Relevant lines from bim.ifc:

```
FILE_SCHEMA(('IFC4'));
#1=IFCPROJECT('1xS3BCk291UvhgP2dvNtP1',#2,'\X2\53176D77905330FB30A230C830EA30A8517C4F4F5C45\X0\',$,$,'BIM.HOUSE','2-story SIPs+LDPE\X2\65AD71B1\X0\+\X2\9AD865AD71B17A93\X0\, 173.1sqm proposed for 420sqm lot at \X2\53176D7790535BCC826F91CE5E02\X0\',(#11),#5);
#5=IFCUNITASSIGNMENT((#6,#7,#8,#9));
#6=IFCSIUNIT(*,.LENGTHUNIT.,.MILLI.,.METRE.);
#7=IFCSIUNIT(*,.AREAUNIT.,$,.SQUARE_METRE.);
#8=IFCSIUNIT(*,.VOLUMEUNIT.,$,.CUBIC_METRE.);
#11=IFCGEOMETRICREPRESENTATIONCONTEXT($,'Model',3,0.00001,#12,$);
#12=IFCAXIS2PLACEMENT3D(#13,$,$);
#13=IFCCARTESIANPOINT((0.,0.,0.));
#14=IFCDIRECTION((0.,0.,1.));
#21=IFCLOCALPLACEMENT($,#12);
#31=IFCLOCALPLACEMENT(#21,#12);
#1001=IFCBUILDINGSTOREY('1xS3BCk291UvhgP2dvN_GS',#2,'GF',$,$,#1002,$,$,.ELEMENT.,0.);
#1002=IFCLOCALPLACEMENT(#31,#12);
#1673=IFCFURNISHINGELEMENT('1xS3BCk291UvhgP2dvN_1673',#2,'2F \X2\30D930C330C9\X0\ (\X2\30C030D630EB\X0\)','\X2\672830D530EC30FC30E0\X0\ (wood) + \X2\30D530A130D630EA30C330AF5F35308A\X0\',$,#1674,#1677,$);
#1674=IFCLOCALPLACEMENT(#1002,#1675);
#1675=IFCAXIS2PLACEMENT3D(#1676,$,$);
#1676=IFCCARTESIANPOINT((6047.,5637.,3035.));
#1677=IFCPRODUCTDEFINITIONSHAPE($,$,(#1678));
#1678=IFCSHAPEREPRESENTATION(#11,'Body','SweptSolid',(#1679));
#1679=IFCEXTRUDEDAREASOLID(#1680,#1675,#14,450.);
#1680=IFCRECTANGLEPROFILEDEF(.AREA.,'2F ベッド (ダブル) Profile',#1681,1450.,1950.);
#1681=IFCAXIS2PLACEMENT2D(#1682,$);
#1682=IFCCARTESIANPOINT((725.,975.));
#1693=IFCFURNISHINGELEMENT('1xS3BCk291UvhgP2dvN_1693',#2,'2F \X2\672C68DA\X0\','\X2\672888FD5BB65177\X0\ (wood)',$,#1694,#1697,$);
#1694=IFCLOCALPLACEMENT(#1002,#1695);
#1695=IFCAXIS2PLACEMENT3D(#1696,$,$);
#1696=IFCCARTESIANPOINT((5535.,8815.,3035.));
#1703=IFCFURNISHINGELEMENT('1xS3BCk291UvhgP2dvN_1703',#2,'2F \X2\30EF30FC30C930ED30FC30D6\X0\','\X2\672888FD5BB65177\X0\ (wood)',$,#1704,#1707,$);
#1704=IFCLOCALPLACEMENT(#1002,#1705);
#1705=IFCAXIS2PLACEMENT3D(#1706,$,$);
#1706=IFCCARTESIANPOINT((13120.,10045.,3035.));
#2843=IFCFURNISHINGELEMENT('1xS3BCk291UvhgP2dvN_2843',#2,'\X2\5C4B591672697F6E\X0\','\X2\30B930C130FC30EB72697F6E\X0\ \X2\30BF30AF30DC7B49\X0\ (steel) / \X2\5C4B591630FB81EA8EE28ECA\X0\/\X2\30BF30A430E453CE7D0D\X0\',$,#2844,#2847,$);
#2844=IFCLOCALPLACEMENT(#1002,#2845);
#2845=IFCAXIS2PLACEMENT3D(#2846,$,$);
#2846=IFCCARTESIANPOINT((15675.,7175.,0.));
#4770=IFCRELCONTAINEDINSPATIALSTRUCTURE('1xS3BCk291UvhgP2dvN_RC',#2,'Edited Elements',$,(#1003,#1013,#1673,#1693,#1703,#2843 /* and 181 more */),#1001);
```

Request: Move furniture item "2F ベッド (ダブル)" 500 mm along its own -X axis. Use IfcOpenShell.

```python
import ifcopenshell
import ifcopenshell.api.geometry
import ifcopenshell.util.placement

model = ifcopenshell.open("bim.ifc")

item = model.by_id(1673)
matrix = ifcopenshell.util.placement.get_local_placement(item.ObjectPlacement)
matrix[:3, 3] -= matrix[:3, 0] * 500.0
ifcopenshell.api.geometry.edit_object_placement(model, product=item, matrix=matrix, is_si=False)

print(ifcopenshell.util.placement.get_local_placement(item.ObjectPlacement).round(3) + 0.0)

model.write("bim_updated.ifc")
```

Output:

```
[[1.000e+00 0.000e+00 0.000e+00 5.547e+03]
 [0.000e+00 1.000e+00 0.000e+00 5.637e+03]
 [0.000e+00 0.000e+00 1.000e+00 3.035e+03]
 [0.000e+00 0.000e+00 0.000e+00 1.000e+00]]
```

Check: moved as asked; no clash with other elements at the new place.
